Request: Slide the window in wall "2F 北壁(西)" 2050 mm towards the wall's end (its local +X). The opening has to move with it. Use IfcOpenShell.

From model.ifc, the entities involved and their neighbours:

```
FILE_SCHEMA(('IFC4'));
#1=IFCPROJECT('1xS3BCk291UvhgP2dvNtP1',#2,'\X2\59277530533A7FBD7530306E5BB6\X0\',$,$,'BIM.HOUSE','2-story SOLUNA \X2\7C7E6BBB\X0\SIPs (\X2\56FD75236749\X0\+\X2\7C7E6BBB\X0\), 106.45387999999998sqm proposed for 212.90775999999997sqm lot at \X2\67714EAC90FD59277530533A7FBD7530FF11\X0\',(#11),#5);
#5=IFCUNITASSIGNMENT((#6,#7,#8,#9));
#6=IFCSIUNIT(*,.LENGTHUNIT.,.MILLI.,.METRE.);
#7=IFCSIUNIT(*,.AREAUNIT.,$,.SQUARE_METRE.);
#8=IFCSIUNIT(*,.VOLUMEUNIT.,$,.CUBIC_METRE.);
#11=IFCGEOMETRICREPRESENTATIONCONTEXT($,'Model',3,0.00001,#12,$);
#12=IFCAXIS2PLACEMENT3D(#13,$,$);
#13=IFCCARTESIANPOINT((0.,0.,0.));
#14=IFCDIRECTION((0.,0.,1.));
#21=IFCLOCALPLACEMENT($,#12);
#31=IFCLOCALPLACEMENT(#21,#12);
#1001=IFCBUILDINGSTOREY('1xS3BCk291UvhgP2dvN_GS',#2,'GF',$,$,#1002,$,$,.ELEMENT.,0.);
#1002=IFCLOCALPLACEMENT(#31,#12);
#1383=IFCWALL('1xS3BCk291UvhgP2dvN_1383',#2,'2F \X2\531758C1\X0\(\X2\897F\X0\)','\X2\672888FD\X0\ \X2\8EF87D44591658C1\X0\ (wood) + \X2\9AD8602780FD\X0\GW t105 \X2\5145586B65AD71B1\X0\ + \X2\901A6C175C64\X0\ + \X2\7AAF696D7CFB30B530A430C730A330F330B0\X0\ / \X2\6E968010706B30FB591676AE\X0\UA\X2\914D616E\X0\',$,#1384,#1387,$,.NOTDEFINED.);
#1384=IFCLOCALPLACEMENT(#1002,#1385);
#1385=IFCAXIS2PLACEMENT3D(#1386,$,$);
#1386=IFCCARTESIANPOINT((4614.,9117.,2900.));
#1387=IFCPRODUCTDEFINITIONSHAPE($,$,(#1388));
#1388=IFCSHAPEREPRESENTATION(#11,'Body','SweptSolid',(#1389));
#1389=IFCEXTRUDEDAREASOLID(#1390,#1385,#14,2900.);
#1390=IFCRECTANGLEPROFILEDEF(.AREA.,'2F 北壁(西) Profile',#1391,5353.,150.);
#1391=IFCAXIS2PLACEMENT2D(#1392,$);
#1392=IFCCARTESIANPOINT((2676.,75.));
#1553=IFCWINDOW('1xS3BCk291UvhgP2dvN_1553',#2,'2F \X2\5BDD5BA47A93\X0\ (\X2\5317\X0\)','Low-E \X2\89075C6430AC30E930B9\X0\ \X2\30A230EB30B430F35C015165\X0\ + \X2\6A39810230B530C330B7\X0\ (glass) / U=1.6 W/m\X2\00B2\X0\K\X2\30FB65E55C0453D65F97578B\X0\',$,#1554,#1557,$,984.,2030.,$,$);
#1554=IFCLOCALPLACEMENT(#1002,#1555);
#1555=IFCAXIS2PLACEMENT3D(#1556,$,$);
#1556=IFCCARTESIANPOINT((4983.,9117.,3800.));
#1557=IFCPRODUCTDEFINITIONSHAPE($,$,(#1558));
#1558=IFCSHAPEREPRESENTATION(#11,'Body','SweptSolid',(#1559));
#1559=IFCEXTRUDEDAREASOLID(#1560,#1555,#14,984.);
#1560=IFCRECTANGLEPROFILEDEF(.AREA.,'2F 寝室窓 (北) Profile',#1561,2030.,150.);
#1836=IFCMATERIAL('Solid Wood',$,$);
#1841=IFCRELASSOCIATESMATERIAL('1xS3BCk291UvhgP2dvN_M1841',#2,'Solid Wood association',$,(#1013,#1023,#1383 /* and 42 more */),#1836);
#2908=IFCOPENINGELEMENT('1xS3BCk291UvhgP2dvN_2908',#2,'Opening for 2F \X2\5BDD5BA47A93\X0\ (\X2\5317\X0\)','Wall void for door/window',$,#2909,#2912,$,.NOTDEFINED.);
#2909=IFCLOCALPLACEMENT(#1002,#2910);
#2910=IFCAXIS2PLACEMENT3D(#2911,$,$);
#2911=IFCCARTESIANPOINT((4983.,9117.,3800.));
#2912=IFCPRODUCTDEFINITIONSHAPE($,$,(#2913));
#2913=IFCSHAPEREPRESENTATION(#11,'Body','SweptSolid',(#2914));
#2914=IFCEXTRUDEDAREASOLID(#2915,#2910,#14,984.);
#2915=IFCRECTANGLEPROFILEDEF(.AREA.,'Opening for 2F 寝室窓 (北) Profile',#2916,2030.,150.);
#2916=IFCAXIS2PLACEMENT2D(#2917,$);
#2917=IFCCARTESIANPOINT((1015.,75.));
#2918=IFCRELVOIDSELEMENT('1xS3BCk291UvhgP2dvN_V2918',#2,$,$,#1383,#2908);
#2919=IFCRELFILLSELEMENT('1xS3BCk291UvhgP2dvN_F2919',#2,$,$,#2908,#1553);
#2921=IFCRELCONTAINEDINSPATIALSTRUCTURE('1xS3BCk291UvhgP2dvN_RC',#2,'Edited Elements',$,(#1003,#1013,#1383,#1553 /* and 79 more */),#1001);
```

```python
import ifcopenshell
import ifcopenshell.api.geometry
import ifcopenshell.util.placement
import ifcopenshell.util.unit

model = ifcopenshell.open("model.ifc")
unit_scale = ifcopenshell.util.unit.calculate_unit_scale(model)

window = model.by_guid("1xS3BCk291UvhgP2dvN_1553")
opening = window.FillsVoids[0].RelatingOpeningElement
wall = opening.VoidsElements[0].RelatingBuildingElement

wall_matrix = ifcopenshell.util.placement.get_local_placement(wall.ObjectPlacement)
shift = wall_matrix[:3, 0] * 2.05 / unit_scale
before = ifcopenshell.util.placement.get_local_placement(window.ObjectPlacement)[:3, 3].copy()

# The window is not placed relative to its opening, so move both.
for product in (opening, window):
    matrix = ifcopenshell.util.placement.get_local_placement(product.ObjectPlacement)
    matrix[:3, 3] += shift
    ifcopenshell.api.geometry.edit_object_placement(model, product=product, matrix=matrix, is_si=False)

after = ifcopenshell.util.placement.get_local_placement(window.ObjectPlacement)[:3, 3]
print("window moved by", (after - before).round(3) + 0.0)

model.write("model_v2.ifc")
```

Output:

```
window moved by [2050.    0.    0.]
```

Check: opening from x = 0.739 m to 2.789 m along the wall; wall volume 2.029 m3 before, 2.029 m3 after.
